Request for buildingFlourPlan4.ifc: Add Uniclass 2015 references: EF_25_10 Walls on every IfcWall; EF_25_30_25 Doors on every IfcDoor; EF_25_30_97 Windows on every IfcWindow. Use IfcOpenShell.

First a look at what the model holds.

```python
import ifcopenshell

model = ifcopenshell.open("buildingFlourPlan4.ifc")
print(model.schema)
print("classifications:", [c.Name for c in model.by_type("IfcClassification")])
for ifc_class in ("IfcDoor", "IfcRoof", "IfcStair", "IfcWall", "IfcWindow"):
    print(ifc_class, len(model.by_type(ifc_class)))
```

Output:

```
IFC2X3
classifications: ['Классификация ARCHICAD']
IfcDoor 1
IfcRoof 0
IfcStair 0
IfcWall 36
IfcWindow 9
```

```python
import ifcopenshell
import ifcopenshell.api.classification

model = ifcopenshell.open("buildingFlourPlan4.ifc")

# IFC2X3 requires Source and Edition and has no link from the project to the system.
system = model.create_entity("IfcClassification", Source="NBS", Edition="2015", Name="Uniclass 2015")

codes = {
    "IfcWall": ("EF_25_10", "Walls"),
    "IfcDoor": ("EF_25_30_25", "Doors"),
    "IfcWindow": ("EF_25_30_97", "Windows"),
}
for ifc_class, (code, name) in codes.items():
    products = model.by_type(ifc_class)
    ifcopenshell.api.classification.add_reference(
        model, products=products, classification=system, identification=code, name=name
    )
    print(code, len(products))

model.write("buildingFlourPlan4_v2.ifc")
```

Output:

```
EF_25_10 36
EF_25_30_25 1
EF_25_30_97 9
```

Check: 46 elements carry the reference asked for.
